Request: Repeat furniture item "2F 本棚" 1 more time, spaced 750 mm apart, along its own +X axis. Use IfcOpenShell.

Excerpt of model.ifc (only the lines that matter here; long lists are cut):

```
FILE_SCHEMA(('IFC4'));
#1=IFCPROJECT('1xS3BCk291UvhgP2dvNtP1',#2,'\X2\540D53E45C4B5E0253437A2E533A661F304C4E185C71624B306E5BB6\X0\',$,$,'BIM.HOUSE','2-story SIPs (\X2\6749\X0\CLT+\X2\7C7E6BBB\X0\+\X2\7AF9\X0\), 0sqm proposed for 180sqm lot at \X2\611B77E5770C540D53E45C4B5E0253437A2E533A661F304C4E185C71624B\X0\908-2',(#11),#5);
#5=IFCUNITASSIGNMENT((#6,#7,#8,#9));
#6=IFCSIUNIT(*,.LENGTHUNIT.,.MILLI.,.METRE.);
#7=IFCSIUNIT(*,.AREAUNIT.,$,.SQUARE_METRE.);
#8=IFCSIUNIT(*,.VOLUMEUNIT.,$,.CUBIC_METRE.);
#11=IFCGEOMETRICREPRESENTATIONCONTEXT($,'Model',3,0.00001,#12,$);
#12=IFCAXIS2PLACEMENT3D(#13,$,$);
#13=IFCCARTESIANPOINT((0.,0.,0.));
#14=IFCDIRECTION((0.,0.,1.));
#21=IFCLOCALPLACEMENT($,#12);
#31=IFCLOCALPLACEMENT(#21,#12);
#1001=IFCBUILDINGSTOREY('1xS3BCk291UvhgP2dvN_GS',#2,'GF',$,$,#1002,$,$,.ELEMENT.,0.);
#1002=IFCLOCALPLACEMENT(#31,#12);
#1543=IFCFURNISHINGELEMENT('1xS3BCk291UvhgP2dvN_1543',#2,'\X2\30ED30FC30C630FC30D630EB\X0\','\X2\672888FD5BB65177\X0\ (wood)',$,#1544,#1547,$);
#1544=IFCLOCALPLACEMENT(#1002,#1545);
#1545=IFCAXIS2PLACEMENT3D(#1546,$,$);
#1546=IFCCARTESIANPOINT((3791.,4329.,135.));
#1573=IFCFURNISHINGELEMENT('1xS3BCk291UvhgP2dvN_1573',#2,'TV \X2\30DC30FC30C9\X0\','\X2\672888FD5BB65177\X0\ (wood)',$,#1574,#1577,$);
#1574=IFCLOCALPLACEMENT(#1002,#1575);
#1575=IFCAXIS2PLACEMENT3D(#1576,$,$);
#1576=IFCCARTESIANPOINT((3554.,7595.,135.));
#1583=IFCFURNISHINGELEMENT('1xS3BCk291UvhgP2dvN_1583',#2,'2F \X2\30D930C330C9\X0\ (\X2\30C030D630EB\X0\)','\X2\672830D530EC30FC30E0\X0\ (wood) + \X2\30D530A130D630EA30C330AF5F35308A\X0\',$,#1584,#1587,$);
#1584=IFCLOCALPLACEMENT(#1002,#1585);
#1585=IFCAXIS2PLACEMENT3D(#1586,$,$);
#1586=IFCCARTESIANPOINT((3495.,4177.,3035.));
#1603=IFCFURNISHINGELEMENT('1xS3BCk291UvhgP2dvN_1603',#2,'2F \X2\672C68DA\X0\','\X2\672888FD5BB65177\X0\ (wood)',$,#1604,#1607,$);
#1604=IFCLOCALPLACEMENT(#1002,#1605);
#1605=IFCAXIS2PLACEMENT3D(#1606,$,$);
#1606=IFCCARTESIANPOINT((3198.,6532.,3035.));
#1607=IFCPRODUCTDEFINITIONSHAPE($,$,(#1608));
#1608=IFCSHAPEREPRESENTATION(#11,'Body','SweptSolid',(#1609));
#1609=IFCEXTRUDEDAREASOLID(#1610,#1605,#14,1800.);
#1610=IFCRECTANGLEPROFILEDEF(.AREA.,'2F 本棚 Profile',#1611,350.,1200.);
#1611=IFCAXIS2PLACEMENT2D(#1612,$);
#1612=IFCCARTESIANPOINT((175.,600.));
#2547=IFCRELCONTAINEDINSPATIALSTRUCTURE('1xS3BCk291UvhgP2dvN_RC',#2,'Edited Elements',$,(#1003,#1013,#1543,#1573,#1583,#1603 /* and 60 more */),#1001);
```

```python
import ifcopenshell
import ifcopenshell.api.geometry
import ifcopenshell.api.root
import ifcopenshell.util.element
import ifcopenshell.util.placement
import ifcopenshell.util.unit

model = ifcopenshell.open("model.ifc")
unit_scale = ifcopenshell.util.unit.calculate_unit_scale(model)


def reuse_history(source, copy):
    """copy_class also copies each property set's owner history, people and application; keep the originals."""
    for rel in copy.IsDefinedBy:
        if rel.is_a("IfcRelDefinesByProperties") and (history := rel.RelatingPropertyDefinition.OwnerHistory):
            rel.RelatingPropertyDefinition.OwnerHistory = source.OwnerHistory
            ifcopenshell.util.element.remove_deep2(model, history)


source = model.by_id(1603)
base = ifcopenshell.util.placement.get_local_placement(source.ObjectPlacement)
step = base[:3, 0] * 0.75 / unit_scale

for i in range(1, 2):
    copy = ifcopenshell.api.root.copy_class(model, product=source)
    copy.Representation = ifcopenshell.util.element.copy_deep(
        model, source.Representation, exclude=["IfcGeometricRepresentationContext", "IfcRepresentationMap"]
    )
    reuse_history(source, copy)
    matrix = base.copy()
    matrix[:3, 3] += i * step
    print("added at", matrix[:3, 3].round(3) + 0.0)
    ifcopenshell.api.geometry.edit_object_placement(model, product=copy, matrix=matrix, is_si=False)

model.write("model_v2.ifc")
```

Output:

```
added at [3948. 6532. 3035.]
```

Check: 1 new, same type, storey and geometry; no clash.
